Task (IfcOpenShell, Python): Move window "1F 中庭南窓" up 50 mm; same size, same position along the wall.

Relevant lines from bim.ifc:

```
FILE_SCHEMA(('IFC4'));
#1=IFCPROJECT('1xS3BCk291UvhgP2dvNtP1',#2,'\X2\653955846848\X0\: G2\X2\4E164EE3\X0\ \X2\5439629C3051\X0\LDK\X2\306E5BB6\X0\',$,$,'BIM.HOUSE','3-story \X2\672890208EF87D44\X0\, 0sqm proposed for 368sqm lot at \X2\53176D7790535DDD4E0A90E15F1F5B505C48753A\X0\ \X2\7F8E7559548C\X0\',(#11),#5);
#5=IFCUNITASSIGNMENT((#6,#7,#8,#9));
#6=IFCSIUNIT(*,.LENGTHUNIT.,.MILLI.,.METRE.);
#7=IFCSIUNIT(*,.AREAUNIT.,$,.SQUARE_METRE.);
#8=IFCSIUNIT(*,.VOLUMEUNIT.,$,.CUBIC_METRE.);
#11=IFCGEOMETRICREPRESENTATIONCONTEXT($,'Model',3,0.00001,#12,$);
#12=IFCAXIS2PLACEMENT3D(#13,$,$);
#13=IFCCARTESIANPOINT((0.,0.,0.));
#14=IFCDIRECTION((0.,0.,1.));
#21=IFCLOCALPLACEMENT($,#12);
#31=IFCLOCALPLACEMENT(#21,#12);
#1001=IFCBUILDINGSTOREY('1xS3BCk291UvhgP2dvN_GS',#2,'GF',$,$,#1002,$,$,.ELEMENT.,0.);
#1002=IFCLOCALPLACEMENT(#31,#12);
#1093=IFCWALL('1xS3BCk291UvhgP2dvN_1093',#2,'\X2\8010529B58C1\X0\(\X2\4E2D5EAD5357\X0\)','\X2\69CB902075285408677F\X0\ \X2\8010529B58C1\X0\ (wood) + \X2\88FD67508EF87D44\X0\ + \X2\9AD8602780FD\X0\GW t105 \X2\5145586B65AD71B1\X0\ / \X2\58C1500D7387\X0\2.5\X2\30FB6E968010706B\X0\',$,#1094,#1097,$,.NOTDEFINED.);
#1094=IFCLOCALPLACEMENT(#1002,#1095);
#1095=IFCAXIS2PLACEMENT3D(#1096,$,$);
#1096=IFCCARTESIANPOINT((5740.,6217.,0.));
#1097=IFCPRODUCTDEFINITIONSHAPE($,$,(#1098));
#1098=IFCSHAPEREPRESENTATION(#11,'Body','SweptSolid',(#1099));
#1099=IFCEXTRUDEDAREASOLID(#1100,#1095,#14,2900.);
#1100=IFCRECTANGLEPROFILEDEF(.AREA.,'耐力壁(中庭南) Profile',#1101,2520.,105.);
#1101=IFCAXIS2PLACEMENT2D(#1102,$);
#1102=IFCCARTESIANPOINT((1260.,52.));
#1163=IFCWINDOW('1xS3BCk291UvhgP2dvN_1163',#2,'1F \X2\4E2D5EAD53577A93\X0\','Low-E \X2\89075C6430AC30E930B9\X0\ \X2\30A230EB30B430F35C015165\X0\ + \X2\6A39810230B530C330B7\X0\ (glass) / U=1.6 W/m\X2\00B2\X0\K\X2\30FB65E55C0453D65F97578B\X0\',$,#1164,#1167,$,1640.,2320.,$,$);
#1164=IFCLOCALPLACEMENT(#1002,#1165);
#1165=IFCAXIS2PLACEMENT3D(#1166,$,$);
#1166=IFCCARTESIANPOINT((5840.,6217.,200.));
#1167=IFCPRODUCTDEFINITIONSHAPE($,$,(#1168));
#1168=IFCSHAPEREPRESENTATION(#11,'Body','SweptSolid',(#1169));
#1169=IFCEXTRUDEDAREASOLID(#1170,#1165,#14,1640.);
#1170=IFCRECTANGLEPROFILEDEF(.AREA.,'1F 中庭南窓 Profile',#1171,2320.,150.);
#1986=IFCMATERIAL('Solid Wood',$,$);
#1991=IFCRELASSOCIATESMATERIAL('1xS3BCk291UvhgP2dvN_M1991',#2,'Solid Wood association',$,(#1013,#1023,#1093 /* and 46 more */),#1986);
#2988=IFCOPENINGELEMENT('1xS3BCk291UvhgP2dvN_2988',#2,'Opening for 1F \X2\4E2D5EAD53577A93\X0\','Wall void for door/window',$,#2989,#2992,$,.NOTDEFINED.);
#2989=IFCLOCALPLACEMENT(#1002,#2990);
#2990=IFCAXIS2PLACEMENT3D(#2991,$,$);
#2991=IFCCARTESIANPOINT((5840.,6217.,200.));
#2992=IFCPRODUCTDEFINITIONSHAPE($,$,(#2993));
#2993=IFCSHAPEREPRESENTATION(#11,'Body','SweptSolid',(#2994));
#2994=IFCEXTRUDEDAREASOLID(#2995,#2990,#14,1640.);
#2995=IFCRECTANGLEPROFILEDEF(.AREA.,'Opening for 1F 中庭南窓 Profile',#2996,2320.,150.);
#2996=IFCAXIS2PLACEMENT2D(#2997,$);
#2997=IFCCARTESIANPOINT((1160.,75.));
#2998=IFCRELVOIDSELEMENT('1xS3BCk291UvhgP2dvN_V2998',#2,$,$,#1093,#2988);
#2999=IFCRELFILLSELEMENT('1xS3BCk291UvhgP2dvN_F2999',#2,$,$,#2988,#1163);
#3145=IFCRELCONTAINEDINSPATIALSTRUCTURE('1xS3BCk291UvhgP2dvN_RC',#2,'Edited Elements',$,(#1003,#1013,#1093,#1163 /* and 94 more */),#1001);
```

```python
import numpy as np
import ifcopenshell
import ifcopenshell.api.geometry
import ifcopenshell.util.placement
import ifcopenshell.util.unit

model = ifcopenshell.open("bim.ifc")
unit_scale = ifcopenshell.util.unit.calculate_unit_scale(model)

window = model.by_guid("1xS3BCk291UvhgP2dvN_1163")
opening = window.FillsVoids[0].RelatingOpeningElement
dz = 0.05 / unit_scale

shift = np.array([0.0, 0.0, dz])
# The window is not placed relative to its opening, so move both.
for product in (opening, window):
    matrix = ifcopenshell.util.placement.get_local_placement(product.ObjectPlacement)
    matrix[:3, 3] += shift
    ifcopenshell.api.geometry.edit_object_placement(model, product=product, matrix=matrix, is_si=False)

print(f"moved by {dz * unit_scale:+.3f} m")

model.write("bim_edited.ifc")
```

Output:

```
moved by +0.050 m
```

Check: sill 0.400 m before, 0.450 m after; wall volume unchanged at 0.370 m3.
